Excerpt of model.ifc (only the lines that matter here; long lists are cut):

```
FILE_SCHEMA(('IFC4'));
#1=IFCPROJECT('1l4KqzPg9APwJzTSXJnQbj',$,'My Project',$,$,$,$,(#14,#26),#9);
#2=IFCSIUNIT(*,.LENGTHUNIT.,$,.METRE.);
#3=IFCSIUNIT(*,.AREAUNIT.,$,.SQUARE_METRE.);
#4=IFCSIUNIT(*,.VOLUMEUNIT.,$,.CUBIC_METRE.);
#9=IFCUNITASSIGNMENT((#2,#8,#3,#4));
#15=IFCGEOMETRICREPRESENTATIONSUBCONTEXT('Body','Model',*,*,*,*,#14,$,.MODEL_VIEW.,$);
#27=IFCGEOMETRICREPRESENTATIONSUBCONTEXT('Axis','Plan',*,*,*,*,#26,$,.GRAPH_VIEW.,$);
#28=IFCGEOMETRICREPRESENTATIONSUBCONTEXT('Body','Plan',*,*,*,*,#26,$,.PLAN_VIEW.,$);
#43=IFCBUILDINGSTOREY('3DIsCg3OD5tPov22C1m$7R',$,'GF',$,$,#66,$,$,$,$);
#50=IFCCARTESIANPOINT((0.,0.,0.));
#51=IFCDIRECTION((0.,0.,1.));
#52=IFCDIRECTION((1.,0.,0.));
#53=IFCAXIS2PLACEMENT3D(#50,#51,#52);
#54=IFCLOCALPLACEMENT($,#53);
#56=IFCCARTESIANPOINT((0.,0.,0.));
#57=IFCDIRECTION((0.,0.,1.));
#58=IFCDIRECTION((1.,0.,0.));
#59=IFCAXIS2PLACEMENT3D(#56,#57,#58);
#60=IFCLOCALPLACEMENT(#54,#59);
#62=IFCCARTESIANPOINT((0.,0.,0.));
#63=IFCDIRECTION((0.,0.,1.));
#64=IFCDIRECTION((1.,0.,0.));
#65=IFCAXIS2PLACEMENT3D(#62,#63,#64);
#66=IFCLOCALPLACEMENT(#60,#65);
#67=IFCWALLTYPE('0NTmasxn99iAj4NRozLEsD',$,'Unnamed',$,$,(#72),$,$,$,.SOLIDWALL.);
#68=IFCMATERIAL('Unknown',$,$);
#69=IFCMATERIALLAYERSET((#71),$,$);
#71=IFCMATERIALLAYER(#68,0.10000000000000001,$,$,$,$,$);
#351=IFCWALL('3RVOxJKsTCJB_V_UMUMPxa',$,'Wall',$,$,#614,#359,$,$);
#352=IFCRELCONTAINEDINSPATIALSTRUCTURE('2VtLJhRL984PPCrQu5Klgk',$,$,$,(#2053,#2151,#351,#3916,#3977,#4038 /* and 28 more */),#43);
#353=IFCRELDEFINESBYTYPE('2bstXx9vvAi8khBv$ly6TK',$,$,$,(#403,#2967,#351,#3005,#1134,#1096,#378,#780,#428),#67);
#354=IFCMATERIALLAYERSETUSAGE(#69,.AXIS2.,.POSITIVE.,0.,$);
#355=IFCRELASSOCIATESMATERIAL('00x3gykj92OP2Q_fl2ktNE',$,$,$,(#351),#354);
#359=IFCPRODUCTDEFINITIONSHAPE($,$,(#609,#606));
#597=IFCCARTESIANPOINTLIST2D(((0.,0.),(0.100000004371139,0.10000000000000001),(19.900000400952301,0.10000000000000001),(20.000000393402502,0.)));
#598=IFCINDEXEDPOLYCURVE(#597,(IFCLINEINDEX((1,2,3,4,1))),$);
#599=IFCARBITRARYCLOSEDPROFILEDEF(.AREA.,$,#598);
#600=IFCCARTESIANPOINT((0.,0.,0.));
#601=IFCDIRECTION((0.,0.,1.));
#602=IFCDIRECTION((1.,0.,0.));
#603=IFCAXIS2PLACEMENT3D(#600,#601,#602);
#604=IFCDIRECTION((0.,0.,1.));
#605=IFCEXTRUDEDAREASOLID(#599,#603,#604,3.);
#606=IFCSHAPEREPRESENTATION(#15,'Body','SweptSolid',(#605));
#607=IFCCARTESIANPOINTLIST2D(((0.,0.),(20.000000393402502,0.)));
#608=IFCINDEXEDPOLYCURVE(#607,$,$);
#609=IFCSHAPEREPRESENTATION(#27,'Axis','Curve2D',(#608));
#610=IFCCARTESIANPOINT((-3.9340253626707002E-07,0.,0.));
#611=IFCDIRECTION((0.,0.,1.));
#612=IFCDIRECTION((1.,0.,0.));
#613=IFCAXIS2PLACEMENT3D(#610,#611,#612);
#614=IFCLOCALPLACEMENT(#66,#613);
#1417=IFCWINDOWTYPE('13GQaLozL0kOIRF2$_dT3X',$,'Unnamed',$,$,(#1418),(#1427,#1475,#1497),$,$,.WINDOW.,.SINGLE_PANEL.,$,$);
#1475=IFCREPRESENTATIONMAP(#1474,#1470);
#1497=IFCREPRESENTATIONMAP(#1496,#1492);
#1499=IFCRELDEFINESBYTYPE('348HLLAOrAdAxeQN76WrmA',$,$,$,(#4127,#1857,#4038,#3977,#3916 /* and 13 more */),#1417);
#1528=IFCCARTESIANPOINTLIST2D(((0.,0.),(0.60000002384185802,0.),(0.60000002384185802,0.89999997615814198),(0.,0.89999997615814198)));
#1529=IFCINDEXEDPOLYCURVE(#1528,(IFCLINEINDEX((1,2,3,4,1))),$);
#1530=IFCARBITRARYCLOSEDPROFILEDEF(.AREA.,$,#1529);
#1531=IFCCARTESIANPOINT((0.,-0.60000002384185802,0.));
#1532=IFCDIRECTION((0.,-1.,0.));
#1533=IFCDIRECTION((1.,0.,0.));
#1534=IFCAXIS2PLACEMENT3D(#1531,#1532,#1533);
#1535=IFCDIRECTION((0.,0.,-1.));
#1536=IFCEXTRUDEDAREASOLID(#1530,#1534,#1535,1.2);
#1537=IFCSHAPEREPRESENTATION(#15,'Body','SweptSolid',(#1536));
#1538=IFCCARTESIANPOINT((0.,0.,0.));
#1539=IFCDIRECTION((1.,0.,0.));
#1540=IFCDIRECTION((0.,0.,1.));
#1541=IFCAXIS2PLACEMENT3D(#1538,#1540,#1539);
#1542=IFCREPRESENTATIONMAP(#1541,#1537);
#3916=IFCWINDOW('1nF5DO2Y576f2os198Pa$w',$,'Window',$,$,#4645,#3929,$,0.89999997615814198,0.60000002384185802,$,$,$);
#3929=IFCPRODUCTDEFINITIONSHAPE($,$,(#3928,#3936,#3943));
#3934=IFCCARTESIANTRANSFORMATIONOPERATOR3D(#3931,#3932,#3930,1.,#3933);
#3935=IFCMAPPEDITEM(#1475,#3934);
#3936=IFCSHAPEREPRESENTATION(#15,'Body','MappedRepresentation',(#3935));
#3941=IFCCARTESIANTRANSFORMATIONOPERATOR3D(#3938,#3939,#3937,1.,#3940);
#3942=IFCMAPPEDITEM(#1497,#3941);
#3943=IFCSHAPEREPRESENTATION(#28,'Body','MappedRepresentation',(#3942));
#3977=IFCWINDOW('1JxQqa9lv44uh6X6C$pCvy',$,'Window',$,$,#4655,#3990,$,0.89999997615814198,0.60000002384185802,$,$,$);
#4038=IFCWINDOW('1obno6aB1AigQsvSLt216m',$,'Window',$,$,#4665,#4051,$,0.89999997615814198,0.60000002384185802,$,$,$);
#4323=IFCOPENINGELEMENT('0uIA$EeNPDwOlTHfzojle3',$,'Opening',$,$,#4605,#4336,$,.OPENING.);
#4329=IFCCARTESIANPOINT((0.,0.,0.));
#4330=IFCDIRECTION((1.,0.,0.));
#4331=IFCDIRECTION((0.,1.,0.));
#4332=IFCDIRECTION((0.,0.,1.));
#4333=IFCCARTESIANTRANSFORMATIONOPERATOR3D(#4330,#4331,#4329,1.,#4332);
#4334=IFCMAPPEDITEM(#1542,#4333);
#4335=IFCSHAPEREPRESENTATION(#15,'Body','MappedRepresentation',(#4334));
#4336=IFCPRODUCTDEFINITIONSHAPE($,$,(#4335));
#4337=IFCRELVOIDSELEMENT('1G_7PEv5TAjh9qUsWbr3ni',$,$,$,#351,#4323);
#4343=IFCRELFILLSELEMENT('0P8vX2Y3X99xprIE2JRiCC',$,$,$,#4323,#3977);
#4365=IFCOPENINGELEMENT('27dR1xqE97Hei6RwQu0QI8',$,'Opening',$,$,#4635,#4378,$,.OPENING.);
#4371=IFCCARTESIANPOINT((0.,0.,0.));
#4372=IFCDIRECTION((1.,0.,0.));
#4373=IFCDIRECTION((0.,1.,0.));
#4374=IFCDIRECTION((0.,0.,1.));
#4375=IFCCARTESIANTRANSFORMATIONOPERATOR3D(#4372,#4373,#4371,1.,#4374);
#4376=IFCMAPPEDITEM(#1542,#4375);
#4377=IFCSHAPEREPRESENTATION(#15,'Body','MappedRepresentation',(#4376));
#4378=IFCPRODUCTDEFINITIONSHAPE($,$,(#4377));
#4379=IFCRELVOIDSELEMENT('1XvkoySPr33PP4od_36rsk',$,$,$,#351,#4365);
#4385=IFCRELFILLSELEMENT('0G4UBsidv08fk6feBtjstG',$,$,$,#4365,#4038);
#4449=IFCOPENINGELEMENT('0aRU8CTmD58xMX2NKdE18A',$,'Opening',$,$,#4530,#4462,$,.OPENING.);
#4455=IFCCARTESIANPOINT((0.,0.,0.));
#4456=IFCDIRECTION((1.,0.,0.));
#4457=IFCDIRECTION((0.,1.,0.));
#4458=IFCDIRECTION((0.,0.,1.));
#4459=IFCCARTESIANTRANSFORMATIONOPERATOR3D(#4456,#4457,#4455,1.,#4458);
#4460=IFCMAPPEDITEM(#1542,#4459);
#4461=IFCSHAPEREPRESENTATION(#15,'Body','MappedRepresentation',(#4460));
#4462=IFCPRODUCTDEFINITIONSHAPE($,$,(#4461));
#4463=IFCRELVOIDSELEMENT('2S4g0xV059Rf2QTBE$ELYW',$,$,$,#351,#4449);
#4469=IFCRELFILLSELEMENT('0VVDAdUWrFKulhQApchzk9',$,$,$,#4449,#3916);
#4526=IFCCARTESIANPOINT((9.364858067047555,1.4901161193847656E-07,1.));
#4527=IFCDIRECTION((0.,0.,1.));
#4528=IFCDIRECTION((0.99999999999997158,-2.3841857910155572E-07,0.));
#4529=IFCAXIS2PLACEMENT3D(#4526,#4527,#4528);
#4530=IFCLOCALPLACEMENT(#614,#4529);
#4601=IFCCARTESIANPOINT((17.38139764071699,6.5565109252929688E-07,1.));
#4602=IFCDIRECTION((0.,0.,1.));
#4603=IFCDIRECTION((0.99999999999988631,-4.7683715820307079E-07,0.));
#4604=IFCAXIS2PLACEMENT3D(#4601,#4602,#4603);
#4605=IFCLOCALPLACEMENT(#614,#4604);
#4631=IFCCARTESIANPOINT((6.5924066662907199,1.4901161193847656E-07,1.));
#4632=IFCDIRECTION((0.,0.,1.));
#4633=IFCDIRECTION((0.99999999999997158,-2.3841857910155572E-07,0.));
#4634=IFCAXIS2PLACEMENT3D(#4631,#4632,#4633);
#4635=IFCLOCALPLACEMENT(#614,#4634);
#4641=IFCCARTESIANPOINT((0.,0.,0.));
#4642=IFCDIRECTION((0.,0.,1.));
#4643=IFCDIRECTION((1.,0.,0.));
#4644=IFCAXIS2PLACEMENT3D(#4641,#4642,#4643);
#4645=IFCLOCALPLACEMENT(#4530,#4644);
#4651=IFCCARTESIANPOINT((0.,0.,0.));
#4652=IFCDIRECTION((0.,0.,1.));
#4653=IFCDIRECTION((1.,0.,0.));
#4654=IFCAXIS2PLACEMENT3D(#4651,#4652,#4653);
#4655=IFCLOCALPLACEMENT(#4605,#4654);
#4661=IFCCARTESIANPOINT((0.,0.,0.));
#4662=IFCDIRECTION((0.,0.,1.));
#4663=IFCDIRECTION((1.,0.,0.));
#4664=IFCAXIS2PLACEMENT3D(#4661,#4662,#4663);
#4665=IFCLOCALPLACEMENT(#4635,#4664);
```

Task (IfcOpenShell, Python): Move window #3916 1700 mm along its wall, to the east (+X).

```python
import ifcopenshell
import ifcopenshell.api.geometry
import ifcopenshell.util.placement
import ifcopenshell.util.unit

model = ifcopenshell.open("model.ifc")
unit_scale = ifcopenshell.util.unit.calculate_unit_scale(model)

window = model.by_guid("1nF5DO2Y576f2os198Pa$w")
opening = window.FillsVoids[0].RelatingOpeningElement
wall = opening.VoidsElements[0].RelatingBuildingElement

wall_matrix = ifcopenshell.util.placement.get_local_placement(wall.ObjectPlacement)
shift = wall_matrix[:3, 0] * 1.7 / unit_scale
before = ifcopenshell.util.placement.get_local_placement(window.ObjectPlacement)[:3, 3].copy()

# The window is placed relative to its opening, so it follows when the opening moves.
matrix = ifcopenshell.util.placement.get_local_placement(opening.ObjectPlacement)
matrix[:3, 3] += shift
ifcopenshell.api.geometry.edit_object_placement(
    model, product=opening, matrix=matrix, is_si=False, should_transform_children=True
)

after = ifcopenshell.util.placement.get_local_placement(window.ObjectPlacement)[:3, 3]
print("window moved by", (after - before).round(3) + 0.0)

model.write("model_edited.ifc")
```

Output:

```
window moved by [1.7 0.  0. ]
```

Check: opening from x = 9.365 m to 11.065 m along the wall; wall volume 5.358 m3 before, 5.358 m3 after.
